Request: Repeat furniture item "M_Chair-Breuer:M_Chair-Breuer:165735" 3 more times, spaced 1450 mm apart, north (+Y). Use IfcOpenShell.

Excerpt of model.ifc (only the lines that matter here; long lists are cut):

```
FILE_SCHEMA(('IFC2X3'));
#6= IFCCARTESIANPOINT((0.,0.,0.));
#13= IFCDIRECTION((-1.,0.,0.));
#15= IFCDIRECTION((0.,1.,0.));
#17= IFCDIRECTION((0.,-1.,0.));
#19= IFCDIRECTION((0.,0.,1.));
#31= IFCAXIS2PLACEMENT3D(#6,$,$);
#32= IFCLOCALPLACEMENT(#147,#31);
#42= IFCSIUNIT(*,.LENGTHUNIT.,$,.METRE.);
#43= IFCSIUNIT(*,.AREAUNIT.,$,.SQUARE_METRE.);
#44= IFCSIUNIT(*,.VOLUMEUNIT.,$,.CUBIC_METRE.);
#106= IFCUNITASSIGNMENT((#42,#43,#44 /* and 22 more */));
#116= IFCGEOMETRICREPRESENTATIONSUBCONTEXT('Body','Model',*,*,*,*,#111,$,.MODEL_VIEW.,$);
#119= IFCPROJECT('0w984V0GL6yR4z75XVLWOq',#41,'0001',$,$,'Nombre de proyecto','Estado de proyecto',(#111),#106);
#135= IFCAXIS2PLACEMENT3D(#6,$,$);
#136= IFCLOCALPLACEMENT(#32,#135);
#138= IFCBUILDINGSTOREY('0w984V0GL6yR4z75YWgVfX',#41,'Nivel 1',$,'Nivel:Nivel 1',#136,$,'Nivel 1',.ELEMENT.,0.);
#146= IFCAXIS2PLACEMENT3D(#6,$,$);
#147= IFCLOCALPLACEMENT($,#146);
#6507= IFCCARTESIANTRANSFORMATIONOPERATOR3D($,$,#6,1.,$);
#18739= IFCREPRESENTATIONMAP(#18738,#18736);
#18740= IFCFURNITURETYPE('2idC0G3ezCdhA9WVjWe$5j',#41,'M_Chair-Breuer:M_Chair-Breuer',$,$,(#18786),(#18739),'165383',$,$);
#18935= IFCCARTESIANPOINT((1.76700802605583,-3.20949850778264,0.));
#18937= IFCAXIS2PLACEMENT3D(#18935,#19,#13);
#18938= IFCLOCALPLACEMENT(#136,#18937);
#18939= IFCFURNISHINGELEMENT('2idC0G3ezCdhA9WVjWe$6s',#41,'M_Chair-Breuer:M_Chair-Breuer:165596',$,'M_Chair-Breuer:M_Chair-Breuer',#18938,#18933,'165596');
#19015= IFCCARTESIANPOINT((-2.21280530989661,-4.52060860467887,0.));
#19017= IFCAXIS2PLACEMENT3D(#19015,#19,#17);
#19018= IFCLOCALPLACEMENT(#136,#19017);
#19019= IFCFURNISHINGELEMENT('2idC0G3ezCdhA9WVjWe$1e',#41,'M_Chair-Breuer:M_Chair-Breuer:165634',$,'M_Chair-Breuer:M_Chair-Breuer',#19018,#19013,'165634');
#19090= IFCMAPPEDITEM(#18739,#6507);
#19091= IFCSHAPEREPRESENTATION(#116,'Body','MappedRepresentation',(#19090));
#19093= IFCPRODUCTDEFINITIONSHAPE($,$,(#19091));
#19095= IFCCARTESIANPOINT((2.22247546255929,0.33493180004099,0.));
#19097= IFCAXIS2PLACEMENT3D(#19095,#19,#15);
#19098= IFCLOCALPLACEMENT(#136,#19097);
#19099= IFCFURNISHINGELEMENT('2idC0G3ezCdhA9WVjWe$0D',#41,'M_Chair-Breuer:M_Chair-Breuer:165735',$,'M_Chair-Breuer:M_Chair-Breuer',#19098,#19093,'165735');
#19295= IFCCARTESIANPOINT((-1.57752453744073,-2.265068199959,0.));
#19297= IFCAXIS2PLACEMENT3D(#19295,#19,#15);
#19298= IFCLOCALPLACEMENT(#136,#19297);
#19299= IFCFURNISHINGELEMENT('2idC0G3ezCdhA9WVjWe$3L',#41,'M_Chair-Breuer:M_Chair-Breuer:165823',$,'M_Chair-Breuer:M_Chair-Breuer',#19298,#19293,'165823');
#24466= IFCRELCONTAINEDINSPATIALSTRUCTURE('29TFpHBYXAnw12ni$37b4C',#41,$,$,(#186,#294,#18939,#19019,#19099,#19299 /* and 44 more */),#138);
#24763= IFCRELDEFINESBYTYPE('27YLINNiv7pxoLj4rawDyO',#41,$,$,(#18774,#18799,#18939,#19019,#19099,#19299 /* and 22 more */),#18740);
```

```python
import numpy as np
import ifcopenshell
import ifcopenshell.api.geometry
import ifcopenshell.api.root
import ifcopenshell.util.element
import ifcopenshell.util.placement

model = ifcopenshell.open("model.ifc")


def reuse_history(source, copy):
    """copy_class also copies each property set's owner history, people and application; keep the originals."""
    for rel in copy.IsDefinedBy:
        if rel.is_a("IfcRelDefinesByProperties") and (history := rel.RelatingPropertyDefinition.OwnerHistory):
            rel.RelatingPropertyDefinition.OwnerHistory = source.OwnerHistory
            ifcopenshell.util.element.remove_deep2(model, history)


source = model.by_id(19099)
base = ifcopenshell.util.placement.get_local_placement(source.ObjectPlacement)
step = np.array([0.0, 1.0, 0.0]) * 1.45

for i in range(1, 4):
    copy = ifcopenshell.api.root.copy_class(model, product=source)
    copy.Representation = ifcopenshell.util.element.copy_deep(
        model, source.Representation, exclude=["IfcGeometricRepresentationContext", "IfcRepresentationMap"]
    )
    copy.Name = "M_Chair-Breuer:M_Chair-Breuer"
    copy.Tag = None
    reuse_history(source, copy)
    matrix = base.copy()
    matrix[:3, 3] += i * step
    print("added at", matrix[:3, 3].round(3) + 0.0)
    ifcopenshell.api.geometry.edit_object_placement(model, product=copy, matrix=matrix, is_si=False)

model.write("model_rev.ifc")
```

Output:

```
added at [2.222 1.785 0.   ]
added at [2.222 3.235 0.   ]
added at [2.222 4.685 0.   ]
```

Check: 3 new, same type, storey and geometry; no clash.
